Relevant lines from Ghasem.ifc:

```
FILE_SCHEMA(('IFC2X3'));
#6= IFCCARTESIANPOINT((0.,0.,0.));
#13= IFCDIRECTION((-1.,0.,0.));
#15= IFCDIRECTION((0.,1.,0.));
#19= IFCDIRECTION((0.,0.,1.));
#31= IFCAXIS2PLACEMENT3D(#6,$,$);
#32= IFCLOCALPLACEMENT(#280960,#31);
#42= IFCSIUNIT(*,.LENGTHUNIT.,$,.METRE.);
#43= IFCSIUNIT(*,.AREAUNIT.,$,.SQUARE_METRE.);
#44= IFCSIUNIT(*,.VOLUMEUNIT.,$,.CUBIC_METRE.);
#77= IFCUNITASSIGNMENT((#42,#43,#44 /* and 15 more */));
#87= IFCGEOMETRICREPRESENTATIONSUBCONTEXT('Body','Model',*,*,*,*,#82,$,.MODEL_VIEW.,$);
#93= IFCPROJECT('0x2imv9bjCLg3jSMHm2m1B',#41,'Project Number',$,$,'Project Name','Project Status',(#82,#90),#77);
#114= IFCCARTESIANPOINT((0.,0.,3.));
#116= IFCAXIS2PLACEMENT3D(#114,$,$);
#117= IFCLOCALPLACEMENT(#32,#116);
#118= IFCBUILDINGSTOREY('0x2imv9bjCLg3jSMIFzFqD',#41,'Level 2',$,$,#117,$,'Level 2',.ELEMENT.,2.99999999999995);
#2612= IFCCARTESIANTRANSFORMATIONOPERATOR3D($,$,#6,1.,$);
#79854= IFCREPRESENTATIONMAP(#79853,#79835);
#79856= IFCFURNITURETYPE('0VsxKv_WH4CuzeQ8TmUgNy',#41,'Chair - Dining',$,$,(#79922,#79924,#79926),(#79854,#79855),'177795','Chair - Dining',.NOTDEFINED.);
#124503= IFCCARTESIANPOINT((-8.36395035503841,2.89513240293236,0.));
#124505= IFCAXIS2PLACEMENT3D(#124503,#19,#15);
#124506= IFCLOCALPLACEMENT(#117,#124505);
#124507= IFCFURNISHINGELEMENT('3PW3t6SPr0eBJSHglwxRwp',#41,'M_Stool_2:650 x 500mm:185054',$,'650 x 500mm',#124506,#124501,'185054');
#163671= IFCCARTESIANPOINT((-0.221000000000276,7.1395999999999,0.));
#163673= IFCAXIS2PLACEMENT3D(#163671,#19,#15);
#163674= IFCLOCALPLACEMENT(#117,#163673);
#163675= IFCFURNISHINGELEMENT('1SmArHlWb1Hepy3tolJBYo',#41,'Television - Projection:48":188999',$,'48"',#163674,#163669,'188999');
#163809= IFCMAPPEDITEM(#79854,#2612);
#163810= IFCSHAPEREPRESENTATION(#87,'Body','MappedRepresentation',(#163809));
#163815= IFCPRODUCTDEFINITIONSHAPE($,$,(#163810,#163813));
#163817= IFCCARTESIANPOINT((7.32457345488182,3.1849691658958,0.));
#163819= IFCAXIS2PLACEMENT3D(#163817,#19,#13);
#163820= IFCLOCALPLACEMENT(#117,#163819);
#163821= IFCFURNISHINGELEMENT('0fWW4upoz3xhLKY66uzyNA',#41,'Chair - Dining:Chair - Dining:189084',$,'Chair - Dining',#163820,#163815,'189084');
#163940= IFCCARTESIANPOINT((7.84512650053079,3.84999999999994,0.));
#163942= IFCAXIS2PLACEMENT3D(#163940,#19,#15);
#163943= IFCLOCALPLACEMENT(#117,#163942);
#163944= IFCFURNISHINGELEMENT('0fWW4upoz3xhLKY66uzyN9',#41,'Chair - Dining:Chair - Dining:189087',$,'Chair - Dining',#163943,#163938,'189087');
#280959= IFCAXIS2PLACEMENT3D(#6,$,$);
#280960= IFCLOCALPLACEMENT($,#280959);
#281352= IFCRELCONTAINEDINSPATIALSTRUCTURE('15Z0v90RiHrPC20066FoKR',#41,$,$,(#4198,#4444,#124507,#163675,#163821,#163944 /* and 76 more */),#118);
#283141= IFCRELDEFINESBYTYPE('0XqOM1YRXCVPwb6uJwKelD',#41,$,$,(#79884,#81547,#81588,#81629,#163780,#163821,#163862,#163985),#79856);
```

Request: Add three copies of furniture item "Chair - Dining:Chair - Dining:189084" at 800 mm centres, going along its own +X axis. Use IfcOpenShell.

```python
import ifcopenshell
import ifcopenshell.api.geometry
import ifcopenshell.api.root
import ifcopenshell.util.element
import ifcopenshell.util.placement
import ifcopenshell.util.unit

model = ifcopenshell.open("Ghasem.ifc")
unit_scale = ifcopenshell.util.unit.calculate_unit_scale(model)


def reuse_history(source, copy):
    """copy_class also copies each property set's owner history, people and application; keep the originals."""
    for rel in copy.IsDefinedBy:
        if rel.is_a("IfcRelDefinesByProperties") and (history := rel.RelatingPropertyDefinition.OwnerHistory):
            rel.RelatingPropertyDefinition.OwnerHistory = source.OwnerHistory
            ifcopenshell.util.element.remove_deep2(model, history)


source = model.by_guid("0fWW4upoz3xhLKY66uzyNA")
base = ifcopenshell.util.placement.get_local_placement(source.ObjectPlacement)
step = base[:3, 0] * 0.8 / unit_scale

for i in range(1, 4):
    copy = ifcopenshell.api.root.copy_class(model, product=source)
    copy.Representation = ifcopenshell.util.element.copy_deep(
        model, source.Representation, exclude=["IfcGeometricRepresentationContext", "IfcRepresentationMap"]
    )
    copy.Name = "Chair - Dining:Chair - Dining"
    copy.Tag = None
    reuse_history(source, copy)
    matrix = base.copy()
    matrix[:3, 3] += i * step
    print("added at", matrix[:3, 3].round(3) + 0.0)
    ifcopenshell.api.geometry.edit_object_placement(model, product=copy, matrix=matrix, is_si=False)

model.write("Ghasem-out.ifc")
```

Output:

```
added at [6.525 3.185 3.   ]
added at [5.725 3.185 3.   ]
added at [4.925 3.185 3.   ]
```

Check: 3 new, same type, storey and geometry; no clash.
